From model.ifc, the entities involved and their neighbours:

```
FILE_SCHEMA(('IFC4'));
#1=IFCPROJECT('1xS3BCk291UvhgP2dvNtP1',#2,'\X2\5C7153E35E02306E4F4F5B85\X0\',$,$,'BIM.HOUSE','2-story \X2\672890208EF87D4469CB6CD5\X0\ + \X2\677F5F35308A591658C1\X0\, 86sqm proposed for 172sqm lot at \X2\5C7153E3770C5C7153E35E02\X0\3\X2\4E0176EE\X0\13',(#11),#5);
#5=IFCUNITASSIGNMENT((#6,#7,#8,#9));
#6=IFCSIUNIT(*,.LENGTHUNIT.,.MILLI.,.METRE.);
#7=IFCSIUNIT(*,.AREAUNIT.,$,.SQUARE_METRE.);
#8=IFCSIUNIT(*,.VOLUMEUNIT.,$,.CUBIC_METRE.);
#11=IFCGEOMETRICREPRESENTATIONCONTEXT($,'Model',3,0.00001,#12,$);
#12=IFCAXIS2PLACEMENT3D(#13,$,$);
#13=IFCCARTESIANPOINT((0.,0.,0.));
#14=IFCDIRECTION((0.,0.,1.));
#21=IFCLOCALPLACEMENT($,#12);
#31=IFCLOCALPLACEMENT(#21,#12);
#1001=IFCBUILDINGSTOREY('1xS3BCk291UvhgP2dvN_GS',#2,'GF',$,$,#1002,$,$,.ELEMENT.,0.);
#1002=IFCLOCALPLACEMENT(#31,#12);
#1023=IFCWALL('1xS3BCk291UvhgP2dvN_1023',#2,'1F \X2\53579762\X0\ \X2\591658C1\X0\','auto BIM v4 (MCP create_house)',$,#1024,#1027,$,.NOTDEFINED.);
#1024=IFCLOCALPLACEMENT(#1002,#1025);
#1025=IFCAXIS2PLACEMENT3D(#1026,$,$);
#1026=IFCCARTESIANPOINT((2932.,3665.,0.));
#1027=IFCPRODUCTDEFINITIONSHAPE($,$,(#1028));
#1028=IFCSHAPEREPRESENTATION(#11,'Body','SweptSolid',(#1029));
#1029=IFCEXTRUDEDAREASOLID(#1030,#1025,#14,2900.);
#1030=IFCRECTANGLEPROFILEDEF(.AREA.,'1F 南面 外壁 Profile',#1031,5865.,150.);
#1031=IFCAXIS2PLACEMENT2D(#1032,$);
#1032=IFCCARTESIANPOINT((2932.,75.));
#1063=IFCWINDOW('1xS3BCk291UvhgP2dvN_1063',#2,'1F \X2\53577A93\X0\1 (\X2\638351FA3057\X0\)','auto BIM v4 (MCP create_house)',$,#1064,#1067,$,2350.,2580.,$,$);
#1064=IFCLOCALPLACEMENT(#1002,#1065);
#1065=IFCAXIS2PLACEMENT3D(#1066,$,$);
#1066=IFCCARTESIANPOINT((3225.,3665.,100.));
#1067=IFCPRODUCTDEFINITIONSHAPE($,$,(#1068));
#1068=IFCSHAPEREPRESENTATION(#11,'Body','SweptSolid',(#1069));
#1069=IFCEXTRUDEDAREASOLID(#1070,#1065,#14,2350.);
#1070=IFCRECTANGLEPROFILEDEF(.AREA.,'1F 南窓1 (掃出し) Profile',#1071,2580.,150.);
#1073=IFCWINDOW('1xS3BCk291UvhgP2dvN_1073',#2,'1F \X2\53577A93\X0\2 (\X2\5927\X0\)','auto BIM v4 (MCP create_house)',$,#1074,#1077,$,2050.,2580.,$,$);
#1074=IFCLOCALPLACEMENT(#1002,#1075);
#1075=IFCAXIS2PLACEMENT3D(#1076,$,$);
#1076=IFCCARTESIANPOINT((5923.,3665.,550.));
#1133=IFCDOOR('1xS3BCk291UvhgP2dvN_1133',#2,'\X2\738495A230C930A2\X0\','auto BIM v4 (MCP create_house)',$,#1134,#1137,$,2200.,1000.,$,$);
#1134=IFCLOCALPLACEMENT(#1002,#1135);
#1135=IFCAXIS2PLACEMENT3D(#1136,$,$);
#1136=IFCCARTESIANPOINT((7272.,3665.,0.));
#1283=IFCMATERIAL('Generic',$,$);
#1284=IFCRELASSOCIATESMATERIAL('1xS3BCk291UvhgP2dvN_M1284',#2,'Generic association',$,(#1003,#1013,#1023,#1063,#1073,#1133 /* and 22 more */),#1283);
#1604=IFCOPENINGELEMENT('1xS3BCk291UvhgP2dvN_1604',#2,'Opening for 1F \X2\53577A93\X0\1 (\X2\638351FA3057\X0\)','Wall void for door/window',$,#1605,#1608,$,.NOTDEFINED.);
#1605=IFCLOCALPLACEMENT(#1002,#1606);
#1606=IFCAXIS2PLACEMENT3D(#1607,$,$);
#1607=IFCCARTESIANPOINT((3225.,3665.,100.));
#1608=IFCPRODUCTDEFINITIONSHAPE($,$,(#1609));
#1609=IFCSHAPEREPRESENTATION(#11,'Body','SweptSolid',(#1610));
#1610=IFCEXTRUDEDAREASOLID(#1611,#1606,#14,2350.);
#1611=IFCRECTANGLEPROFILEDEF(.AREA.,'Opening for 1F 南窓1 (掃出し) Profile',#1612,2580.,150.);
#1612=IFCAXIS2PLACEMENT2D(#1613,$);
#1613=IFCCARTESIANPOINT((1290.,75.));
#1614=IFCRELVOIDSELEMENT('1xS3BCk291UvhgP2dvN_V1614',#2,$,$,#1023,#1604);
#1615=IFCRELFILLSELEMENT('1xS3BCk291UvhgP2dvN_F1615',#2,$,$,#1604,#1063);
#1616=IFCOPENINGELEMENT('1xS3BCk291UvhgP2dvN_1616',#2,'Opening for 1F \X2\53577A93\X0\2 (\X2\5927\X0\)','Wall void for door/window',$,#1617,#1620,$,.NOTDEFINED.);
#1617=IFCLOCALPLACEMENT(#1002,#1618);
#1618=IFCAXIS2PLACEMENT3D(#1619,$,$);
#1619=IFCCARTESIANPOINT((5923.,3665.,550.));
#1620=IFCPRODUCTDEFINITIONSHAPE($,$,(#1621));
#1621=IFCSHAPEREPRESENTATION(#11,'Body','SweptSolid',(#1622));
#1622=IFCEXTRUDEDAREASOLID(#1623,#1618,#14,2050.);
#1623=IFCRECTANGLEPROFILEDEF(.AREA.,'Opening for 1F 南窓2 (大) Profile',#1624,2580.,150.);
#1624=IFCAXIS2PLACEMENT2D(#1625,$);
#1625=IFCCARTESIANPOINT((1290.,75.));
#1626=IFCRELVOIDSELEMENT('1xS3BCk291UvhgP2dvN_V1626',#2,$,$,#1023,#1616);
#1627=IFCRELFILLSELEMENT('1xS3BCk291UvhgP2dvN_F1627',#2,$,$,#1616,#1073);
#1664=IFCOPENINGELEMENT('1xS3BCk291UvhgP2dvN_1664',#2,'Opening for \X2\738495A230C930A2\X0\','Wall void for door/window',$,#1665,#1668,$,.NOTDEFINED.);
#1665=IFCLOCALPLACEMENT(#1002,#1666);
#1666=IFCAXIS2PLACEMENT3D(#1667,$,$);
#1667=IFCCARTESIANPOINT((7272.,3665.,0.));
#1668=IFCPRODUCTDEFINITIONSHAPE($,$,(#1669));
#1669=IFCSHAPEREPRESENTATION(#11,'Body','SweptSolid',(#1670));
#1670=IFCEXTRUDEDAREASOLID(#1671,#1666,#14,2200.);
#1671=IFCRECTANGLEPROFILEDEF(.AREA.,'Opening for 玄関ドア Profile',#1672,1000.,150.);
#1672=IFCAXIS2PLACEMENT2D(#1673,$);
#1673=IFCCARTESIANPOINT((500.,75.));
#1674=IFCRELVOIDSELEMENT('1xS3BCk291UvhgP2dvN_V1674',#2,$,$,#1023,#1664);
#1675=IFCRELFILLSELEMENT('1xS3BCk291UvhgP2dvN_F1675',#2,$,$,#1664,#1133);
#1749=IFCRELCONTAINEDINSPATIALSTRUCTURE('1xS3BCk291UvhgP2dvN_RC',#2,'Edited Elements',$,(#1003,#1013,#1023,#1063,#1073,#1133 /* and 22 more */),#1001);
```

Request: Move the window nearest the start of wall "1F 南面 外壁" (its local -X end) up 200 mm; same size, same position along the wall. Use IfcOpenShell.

```python
import numpy as np
import ifcopenshell
import ifcopenshell.api.geometry
import ifcopenshell.util.placement
import ifcopenshell.util.unit

model = ifcopenshell.open("model.ifc")
unit_scale = ifcopenshell.util.unit.calculate_unit_scale(model)

window = model.by_guid("1xS3BCk291UvhgP2dvN_1063")
opening = window.FillsVoids[0].RelatingOpeningElement
dz = 0.2 / unit_scale

shift = np.array([0.0, 0.0, dz])
# The window is not placed relative to its opening, so move both.
for product in (opening, window):
    matrix = ifcopenshell.util.placement.get_local_placement(product.ObjectPlacement)
    matrix[:3, 3] += shift
    ifcopenshell.api.geometry.edit_object_placement(model, product=product, matrix=matrix, is_si=False)

print(f"moved by {dz * unit_scale:+.3f} m")

model.write("model-out.ifc")
```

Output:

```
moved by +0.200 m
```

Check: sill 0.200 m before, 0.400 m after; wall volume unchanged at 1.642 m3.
